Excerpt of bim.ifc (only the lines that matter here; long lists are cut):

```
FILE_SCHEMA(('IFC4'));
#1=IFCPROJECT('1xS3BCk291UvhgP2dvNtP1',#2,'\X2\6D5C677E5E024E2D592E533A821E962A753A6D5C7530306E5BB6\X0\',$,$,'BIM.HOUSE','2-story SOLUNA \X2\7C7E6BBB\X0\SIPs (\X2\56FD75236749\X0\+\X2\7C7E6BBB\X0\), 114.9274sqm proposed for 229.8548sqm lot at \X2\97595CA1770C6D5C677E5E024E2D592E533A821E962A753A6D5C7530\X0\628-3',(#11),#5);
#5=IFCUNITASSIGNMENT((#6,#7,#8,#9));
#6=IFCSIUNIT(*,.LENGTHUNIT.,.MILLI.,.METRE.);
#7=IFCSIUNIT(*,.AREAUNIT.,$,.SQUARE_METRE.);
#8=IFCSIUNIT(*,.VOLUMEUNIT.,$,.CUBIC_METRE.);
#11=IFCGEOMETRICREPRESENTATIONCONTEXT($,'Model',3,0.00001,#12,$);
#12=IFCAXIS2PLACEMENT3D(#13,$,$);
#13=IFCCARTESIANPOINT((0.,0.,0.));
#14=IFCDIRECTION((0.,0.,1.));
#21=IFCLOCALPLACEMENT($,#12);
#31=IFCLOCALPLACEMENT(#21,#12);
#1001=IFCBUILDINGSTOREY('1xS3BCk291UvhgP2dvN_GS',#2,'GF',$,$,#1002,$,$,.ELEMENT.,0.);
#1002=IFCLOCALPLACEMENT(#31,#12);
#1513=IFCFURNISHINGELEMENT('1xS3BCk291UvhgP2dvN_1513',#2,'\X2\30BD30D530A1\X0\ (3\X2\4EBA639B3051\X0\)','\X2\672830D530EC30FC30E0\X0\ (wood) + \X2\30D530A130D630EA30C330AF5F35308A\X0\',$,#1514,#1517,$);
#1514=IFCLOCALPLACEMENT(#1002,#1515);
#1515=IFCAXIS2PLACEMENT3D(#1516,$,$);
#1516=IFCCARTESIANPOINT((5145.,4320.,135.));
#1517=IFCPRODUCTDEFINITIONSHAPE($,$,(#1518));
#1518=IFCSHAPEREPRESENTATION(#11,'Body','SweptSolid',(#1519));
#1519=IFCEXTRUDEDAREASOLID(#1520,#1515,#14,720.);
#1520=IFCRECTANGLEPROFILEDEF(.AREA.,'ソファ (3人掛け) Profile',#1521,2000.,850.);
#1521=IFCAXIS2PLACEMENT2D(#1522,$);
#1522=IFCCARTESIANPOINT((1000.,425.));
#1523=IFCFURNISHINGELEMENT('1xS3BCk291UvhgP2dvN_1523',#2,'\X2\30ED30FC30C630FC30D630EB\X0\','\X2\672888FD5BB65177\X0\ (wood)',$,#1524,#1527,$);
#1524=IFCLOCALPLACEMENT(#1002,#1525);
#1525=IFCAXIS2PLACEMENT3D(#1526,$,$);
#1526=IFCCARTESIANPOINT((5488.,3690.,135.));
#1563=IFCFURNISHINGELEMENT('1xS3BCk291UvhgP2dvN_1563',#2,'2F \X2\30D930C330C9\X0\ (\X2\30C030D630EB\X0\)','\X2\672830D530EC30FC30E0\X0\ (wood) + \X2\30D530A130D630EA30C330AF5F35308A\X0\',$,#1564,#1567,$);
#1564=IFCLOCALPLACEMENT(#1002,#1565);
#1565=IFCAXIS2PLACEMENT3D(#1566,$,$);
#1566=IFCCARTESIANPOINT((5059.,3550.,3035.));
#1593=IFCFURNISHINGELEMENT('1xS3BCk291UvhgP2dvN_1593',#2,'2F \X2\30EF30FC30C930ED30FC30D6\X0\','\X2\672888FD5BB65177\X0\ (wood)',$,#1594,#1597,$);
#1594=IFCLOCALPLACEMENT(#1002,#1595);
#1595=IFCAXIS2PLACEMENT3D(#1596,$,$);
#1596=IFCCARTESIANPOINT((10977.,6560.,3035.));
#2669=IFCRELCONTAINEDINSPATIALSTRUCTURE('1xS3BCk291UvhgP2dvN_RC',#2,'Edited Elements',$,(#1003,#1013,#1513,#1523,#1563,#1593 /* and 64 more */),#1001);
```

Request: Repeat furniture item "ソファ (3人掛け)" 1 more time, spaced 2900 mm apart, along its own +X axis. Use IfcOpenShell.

```python
import ifcopenshell
import ifcopenshell.api.geometry
import ifcopenshell.api.root
import ifcopenshell.util.element
import ifcopenshell.util.placement

model = ifcopenshell.open("bim.ifc")


def reuse_history(source, copy):
    """copy_class also copies each property set's owner history, people and application; keep the originals."""
    for rel in copy.IsDefinedBy:
        if rel.is_a("IfcRelDefinesByProperties") and (history := rel.RelatingPropertyDefinition.OwnerHistory):
            rel.RelatingPropertyDefinition.OwnerHistory = source.OwnerHistory
            ifcopenshell.util.element.remove_deep2(model, history)


source = model.by_id(1513)
base = ifcopenshell.util.placement.get_local_placement(source.ObjectPlacement)
step = base[:3, 0] * 2900.0

for i in range(1, 2):
    copy = ifcopenshell.api.root.copy_class(model, product=source)
    copy.Representation = ifcopenshell.util.element.copy_deep(
        model, source.Representation, exclude=["IfcGeometricRepresentationContext", "IfcRepresentationMap"]
    )
    reuse_history(source, copy)
    matrix = base.copy()
    matrix[:3, 3] += i * step
    print("added at", matrix[:3, 3].round(3) + 0.0)
    ifcopenshell.api.geometry.edit_object_placement(model, product=copy, matrix=matrix, is_si=False)

model.write("bim_rev.ifc")
```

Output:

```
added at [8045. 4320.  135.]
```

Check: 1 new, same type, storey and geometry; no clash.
